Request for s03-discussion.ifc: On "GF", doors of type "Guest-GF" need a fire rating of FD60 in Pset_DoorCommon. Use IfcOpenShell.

First a look at what the model holds.

```python
import ifcopenshell
import ifcopenshell.util.element

model = ifcopenshell.open("s03-discussion.ifc")
print(model.schema)
storey = next(s for s in model.by_type("IfcBuildingStorey") if s.Name == "GF")
doors = [e for e in ifcopenshell.util.element.get_decomposition(storey) if e.is_a("IfcDoor")]
seen = {}
for e in doors:
    element_type = ifcopenshell.util.element.get_type(e)
    key = (element_type.Name if element_type != e and element_type else None, ifcopenshell.util.element.get_pset(e, "Pset_DoorCommon", "FireRating"))
    seen[key] = seen.get(key, 0) + 1
for (name, value), count in sorted(seen.items(), key=str):
    print(count, "x", name, "|", value)
```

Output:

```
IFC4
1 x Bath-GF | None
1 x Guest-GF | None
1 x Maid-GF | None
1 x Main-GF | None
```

```python
import ifcopenshell
import ifcopenshell.api.pset
import ifcopenshell.util.element

model = ifcopenshell.open("s03-discussion.ifc")

storey = next(s for s in model.by_type("IfcBuildingStorey") if s.Name == "GF")
doors = [e for e in ifcopenshell.util.element.get_decomposition(storey) if e.is_a("IfcDoor")]

count = 0
for e in doors:
    element_type = ifcopenshell.util.element.get_type(e)
    if element_type in (None, e) or element_type.Name != "Guest-GF":
        continue
    # add_pset returns the element's existing set when there is one.
    pset = ifcopenshell.api.pset.add_pset(model, product=e, name="Pset_DoorCommon")
    ifcopenshell.api.pset.edit_pset(model, pset=pset, properties={"FireRating": "FD60"})
    count += 1

print(count, "doors updated")

model.write("s03-discussion_updated.ifc")
```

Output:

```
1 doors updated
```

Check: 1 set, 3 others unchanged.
